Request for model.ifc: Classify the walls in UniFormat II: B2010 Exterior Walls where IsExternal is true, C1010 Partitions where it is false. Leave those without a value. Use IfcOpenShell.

First a look at what the model holds.

```python
import ifcopenshell
import ifcopenshell.util.element

model = ifcopenshell.open("model.ifc")
print(model.schema)
print("classifications:", [c.Name for c in model.by_type("IfcClassification")])
values = [ifcopenshell.util.element.get_pset(e, "Pset_WallCommon", "IsExternal") for e in model.by_type("IfcWall")]
for value in (True, False, None):
    print("IsExternal", value, values.count(value))
```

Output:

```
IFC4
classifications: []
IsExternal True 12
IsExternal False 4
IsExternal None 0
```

```python
import ifcopenshell
import ifcopenshell.api.classification
import ifcopenshell.util.element

model = ifcopenshell.open("model.ifc")

system = ifcopenshell.api.classification.add_classification(model, classification="UniFormat II")

walls = model.by_type("IfcWall")
external = {e: ifcopenshell.util.element.get_pset(e, "Pset_WallCommon", "IsExternal") for e in walls}
for flag, code, name in ((True, "B2010", "Exterior Walls"), (False, "C1010", "Partitions")):
    products = [e for e in walls if external[e] is flag]
    ifcopenshell.api.classification.add_reference(
        model, products=products, classification=system, identification=code, name=name
    )
    print(code, len(products))

model.write("model_v2.ifc")
```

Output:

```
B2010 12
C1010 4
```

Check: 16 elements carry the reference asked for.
